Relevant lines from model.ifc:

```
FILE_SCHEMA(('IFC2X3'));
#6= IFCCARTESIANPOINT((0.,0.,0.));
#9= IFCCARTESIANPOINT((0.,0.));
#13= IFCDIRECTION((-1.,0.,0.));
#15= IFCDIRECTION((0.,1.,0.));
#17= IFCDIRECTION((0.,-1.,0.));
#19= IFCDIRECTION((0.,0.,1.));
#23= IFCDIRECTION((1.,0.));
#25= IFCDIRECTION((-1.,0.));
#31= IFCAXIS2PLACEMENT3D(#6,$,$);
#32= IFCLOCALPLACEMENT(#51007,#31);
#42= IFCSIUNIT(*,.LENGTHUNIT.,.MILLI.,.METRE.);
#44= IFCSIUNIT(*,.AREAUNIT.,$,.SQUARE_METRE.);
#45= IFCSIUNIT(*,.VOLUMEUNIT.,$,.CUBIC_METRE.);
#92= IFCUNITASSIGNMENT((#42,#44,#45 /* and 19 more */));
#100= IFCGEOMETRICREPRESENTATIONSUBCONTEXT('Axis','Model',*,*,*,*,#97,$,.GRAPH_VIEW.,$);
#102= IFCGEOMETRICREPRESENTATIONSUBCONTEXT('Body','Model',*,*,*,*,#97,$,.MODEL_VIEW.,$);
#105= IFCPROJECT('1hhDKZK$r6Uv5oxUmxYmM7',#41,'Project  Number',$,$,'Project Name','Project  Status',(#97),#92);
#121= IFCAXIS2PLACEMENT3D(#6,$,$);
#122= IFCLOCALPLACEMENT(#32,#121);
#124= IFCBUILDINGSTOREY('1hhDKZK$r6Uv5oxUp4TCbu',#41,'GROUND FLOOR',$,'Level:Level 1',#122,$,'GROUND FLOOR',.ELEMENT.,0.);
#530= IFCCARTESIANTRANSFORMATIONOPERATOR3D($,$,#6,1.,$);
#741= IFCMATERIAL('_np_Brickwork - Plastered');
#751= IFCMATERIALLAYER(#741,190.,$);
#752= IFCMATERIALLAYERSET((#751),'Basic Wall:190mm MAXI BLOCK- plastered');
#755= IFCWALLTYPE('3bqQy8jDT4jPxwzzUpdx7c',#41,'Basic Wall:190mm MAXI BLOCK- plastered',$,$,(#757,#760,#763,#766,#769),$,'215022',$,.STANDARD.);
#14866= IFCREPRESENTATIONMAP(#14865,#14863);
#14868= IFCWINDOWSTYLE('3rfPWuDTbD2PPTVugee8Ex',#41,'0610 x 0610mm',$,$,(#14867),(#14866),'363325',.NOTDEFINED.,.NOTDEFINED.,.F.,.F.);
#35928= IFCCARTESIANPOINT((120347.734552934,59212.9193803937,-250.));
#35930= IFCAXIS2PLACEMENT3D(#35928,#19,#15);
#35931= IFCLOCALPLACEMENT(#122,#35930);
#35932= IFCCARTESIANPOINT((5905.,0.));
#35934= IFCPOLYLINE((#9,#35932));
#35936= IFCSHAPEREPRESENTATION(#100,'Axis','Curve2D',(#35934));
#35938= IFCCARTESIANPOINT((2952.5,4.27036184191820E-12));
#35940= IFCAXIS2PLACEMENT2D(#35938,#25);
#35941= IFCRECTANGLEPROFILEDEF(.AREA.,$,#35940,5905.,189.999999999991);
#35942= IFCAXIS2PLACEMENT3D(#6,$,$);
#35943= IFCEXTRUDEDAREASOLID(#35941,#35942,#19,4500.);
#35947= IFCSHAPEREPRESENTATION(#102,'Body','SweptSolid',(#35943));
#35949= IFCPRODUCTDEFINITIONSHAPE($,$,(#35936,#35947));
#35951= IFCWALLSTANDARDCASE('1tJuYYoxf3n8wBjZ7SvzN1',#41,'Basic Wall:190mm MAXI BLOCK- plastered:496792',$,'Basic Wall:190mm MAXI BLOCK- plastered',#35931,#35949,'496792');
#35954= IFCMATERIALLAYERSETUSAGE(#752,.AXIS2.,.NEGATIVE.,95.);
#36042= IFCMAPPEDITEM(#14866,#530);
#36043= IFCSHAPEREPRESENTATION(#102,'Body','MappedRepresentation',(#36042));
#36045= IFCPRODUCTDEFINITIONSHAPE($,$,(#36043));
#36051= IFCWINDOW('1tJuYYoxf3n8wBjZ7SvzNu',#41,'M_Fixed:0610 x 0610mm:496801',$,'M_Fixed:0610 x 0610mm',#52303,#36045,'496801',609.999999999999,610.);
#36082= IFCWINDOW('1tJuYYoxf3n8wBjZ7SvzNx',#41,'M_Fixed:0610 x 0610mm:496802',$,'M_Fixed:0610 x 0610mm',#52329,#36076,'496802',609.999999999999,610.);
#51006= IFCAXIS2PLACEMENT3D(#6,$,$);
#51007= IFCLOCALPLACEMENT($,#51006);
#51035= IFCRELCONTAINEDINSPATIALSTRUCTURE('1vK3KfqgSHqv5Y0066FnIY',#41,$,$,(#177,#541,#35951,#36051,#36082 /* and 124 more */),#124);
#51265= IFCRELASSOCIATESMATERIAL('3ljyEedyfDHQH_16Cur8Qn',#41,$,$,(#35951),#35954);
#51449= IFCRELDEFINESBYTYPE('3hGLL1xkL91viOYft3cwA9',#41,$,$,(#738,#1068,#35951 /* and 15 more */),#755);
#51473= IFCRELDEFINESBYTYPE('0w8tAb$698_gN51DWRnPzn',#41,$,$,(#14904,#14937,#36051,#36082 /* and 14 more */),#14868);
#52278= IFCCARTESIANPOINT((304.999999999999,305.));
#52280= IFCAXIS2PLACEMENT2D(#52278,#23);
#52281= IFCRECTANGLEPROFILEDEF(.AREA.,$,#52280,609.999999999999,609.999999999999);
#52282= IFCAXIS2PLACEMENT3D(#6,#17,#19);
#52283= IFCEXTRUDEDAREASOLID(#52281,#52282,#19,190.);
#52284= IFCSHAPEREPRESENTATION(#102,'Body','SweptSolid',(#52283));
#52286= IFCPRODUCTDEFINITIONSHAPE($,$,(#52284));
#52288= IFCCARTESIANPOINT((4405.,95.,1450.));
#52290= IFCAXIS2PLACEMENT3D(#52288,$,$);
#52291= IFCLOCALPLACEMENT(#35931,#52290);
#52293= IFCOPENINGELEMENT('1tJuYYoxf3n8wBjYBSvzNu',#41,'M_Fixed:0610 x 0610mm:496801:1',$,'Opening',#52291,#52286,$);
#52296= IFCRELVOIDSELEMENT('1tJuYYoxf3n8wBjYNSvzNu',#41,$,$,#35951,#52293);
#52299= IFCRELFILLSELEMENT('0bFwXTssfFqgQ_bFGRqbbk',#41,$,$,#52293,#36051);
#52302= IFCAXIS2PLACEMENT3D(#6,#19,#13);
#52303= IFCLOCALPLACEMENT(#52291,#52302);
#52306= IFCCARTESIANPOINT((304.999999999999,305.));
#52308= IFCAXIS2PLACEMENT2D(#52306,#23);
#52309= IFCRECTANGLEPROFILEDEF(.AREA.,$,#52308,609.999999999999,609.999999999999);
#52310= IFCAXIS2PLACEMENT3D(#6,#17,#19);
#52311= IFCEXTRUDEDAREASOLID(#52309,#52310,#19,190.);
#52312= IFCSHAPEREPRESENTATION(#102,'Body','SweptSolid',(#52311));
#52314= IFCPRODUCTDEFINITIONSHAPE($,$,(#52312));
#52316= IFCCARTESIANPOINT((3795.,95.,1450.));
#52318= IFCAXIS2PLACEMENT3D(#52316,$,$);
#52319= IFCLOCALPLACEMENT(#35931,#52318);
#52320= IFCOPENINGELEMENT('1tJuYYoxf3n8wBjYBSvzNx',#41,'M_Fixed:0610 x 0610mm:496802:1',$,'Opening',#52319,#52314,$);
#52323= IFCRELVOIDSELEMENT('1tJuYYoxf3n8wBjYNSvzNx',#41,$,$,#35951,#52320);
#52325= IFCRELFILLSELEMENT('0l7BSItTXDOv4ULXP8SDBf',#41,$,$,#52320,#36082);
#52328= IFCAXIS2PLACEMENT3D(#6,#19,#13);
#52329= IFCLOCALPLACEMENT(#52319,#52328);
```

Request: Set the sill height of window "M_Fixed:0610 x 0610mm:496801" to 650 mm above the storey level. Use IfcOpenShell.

```python
import numpy as np
import ifcopenshell
import ifcopenshell.api.geometry
import ifcopenshell.geom
import ifcopenshell.util.element
import ifcopenshell.util.placement
import ifcopenshell.util.shape
import ifcopenshell.util.unit

model = ifcopenshell.open("model.ifc")
unit_scale = ifcopenshell.util.unit.calculate_unit_scale(model)

window = model.by_id(36051)
opening = window.FillsVoids[0].RelatingOpeningElement
storey = ifcopenshell.util.element.get_container(window, ifc_class="IfcBuildingStorey")
level = ifcopenshell.util.placement.get_local_placement(storey.ObjectPlacement)[2, 3]

# The opening's origin need not be at the sill, so measure its lowest point.
shape = ifcopenshell.geom.create_shape(ifcopenshell.geom.settings(), opening)
bottom = ifcopenshell.util.shape.get_shape_bottom_elevation(shape, shape.geometry) / unit_scale
dz = level + 0.65 / unit_scale - bottom

shift = np.array([0.0, 0.0, dz])
# The window is placed relative to its opening, so it follows when the opening moves.
matrix = ifcopenshell.util.placement.get_local_placement(opening.ObjectPlacement)
matrix[:3, 3] += shift
ifcopenshell.api.geometry.edit_object_placement(
    model, product=opening, matrix=matrix, is_si=False, should_transform_children=True
)

print(f"moved by {dz * unit_scale:+.3f} m")

model.write("model_edited.ifc")
```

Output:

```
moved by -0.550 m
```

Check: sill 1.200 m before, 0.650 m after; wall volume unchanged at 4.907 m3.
